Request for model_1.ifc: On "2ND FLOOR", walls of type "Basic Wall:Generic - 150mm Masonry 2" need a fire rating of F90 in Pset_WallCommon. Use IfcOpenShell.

First a look at what the model holds.

```python
import ifcopenshell
import ifcopenshell.util.element

model = ifcopenshell.open("model_1.ifc")
print(model.schema)
storey = next(s for s in model.by_type("IfcBuildingStorey") if s.Name == "2ND FLOOR")
walls = [e for e in ifcopenshell.util.element.get_decomposition(storey) if e.is_a("IfcWall")]
seen = {}
for e in walls:
    element_type = ifcopenshell.util.element.get_type(e)
    key = (element_type.Name if element_type != e and element_type else None, ifcopenshell.util.element.get_pset(e, "Pset_WallCommon", "FireRating"))
    seen[key] = seen.get(key, 0) + 1
for (name, value), count in sorted(seen.items(), key=str):
    print(count, "x", name, "|", value)
```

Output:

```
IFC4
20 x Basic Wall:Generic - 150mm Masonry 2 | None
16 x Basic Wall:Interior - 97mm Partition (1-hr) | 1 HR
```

```python
import ifcopenshell
import ifcopenshell.api.pset
import ifcopenshell.util.element

model = ifcopenshell.open("model_1.ifc")

storey = next(s for s in model.by_type("IfcBuildingStorey") if s.Name == "2ND FLOOR")
walls = [e for e in ifcopenshell.util.element.get_decomposition(storey) if e.is_a("IfcWall")]

count = 0
for e in walls:
    element_type = ifcopenshell.util.element.get_type(e)
    if element_type in (None, e) or element_type.Name != "Basic Wall:Generic - 150mm Masonry 2":
        continue
    # add_pset returns the element's existing set when there is one.
    pset = ifcopenshell.api.pset.add_pset(model, product=e, name="Pset_WallCommon")
    ifcopenshell.api.pset.edit_pset(model, pset=pset, properties={"FireRating": "F90"})
    count += 1

print(count, "walls updated")

model.write("model_1_edited.ifc")
```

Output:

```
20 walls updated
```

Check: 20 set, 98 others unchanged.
